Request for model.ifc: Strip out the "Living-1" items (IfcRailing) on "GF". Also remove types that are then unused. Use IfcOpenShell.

First a look at what the model holds.

```python
import ifcopenshell
import ifcopenshell.util.element

model = ifcopenshell.open("model.ifc")
print(model.schema)
storey = next(s for s in model.by_type("IfcBuildingStorey") if s.Name == "GF")
railings = [e for e in ifcopenshell.util.element.get_decomposition(storey) if e.is_a("IfcRailing")]
seen = {}
for e in railings:
    element_type = ifcopenshell.util.element.get_type(e)
    name = element_type.Name if element_type not in (None, e) else None
    seen[name] = seen.get(name, 0) + 1
for name, count in sorted(seen.items(), key=str):
    print(count, "x", name)
```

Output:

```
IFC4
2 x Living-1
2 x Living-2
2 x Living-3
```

```python
import ifcopenshell
import ifcopenshell.api.root
import ifcopenshell.util.element

model = ifcopenshell.open("model.ifc")

storey = next(s for s in model.by_type("IfcBuildingStorey") if s.Name == "GF")
railings = [e for e in ifcopenshell.util.element.get_decomposition(storey) if e.is_a("IfcRailing")]
targets = [e for e in railings if (t := ifcopenshell.util.element.get_type(e)) not in (None, e) and t.Name == "Living-1"]
types = {ifcopenshell.util.element.get_type(e) for e in targets} - {None, *targets}

for e in targets:
    ifcopenshell.api.root.remove_product(model, product=e)
print(len(targets), "removed")

unused = [t for t in types if not ifcopenshell.util.element.get_types(t)]
for t in unused:
    ifcopenshell.api.root.remove_product(model, product=t)
print(len(unused), "unused types removed")

model.write("model_v2.ifc")
```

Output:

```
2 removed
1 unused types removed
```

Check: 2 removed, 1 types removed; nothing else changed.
